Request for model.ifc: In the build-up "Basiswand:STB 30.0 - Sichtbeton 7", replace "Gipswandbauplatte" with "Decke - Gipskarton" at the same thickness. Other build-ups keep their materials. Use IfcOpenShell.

First a look at what the model holds.

```python
import ifcopenshell
import ifcopenshell.util.element

model = ifcopenshell.open("model.ifc")
print(model.schema)
for layer_set in model.by_type("IfcMaterialLayerSet"):
    if layer_set.LayerSetName == "Basiswand:STB 30.0 - Sichtbeton 7":
        for layer in layer_set.MaterialLayers:
            print(layer.id(), layer.Material and layer.Material.Name, layer.LayerThickness, sep=" | ")
        print(len(ifcopenshell.util.element.get_elements_by_material(model, layer_set)), "elements and types use it")
print(sorted(m.Name for m in model.by_type("IfcMaterial") if m.Name)[:60])
```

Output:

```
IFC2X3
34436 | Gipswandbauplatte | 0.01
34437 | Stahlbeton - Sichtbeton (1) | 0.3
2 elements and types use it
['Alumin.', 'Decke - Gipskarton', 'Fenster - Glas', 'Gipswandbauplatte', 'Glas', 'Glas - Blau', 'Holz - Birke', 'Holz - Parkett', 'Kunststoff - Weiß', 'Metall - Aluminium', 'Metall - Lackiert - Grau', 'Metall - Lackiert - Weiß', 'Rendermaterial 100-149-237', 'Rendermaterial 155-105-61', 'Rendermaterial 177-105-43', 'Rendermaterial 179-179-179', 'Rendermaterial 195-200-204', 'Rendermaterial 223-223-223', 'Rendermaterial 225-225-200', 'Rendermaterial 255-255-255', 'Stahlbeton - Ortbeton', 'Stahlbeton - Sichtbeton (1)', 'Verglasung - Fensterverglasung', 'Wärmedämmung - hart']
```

```python
import ifcopenshell
import ifcopenshell.api.material

model = ifcopenshell.open("model.ifc")

layer_set = next(s for s in model.by_type("IfcMaterialLayerSet") if s.LayerSetName == "Basiswand:STB 30.0 - Sichtbeton 7")
layer = next(l for l in layer_set.MaterialLayers if l.Material and l.Material.Name == "Gipswandbauplatte")
material = next(m for m in model.by_type("IfcMaterial") if m.Name == "Decke - Gipskarton")

# Point this one layer at the other material; renaming the old one would change it everywhere.
ifcopenshell.api.material.edit_layer(model, layer=layer, attributes={}, material=material)

print([l.Material.Name if l.Material else None for l in layer_set.MaterialLayers])

model.write("model_rev.ifc")
```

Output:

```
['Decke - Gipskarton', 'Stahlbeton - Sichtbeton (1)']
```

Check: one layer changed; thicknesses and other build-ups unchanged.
